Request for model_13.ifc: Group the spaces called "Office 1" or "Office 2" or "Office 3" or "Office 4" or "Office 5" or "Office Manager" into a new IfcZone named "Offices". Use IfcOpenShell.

First a look at what the model holds.

```python
import ifcopenshell

model = ifcopenshell.open("model_13.ifc")
print(model.schema)
seen = {}
for space in model.by_type("IfcSpace"):
    seen[space.LongName] = seen.get(space.LongName, 0) + 1
for name, count in sorted(seen.items(), key=str):
    print(count, "x", name)
print("zones:", [z.Name for z in model.by_type("IfcZone")][:20])
```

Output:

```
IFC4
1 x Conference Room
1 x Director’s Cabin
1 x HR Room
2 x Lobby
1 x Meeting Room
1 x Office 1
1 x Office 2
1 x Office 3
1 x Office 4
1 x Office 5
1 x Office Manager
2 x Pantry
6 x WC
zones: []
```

```python
import ifcopenshell
import ifcopenshell.api.group
import ifcopenshell.api.root

model = ifcopenshell.open("model_13.ifc")

names = {"Office 1", "Office 2", "Office 3", "Office 4", "Office 5", "Office Manager"}
spaces = [s for s in model.by_type("IfcSpace") if s.LongName in names]

zone = ifcopenshell.api.root.create_entity(model, ifc_class="IfcZone", name="Offices")
ifcopenshell.api.group.assign_group(model, products=spaces, group=zone)
print(len(spaces), "spaces in", zone.Name)

model.write("model_13_v2.ifc")
```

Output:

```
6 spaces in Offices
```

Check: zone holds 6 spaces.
